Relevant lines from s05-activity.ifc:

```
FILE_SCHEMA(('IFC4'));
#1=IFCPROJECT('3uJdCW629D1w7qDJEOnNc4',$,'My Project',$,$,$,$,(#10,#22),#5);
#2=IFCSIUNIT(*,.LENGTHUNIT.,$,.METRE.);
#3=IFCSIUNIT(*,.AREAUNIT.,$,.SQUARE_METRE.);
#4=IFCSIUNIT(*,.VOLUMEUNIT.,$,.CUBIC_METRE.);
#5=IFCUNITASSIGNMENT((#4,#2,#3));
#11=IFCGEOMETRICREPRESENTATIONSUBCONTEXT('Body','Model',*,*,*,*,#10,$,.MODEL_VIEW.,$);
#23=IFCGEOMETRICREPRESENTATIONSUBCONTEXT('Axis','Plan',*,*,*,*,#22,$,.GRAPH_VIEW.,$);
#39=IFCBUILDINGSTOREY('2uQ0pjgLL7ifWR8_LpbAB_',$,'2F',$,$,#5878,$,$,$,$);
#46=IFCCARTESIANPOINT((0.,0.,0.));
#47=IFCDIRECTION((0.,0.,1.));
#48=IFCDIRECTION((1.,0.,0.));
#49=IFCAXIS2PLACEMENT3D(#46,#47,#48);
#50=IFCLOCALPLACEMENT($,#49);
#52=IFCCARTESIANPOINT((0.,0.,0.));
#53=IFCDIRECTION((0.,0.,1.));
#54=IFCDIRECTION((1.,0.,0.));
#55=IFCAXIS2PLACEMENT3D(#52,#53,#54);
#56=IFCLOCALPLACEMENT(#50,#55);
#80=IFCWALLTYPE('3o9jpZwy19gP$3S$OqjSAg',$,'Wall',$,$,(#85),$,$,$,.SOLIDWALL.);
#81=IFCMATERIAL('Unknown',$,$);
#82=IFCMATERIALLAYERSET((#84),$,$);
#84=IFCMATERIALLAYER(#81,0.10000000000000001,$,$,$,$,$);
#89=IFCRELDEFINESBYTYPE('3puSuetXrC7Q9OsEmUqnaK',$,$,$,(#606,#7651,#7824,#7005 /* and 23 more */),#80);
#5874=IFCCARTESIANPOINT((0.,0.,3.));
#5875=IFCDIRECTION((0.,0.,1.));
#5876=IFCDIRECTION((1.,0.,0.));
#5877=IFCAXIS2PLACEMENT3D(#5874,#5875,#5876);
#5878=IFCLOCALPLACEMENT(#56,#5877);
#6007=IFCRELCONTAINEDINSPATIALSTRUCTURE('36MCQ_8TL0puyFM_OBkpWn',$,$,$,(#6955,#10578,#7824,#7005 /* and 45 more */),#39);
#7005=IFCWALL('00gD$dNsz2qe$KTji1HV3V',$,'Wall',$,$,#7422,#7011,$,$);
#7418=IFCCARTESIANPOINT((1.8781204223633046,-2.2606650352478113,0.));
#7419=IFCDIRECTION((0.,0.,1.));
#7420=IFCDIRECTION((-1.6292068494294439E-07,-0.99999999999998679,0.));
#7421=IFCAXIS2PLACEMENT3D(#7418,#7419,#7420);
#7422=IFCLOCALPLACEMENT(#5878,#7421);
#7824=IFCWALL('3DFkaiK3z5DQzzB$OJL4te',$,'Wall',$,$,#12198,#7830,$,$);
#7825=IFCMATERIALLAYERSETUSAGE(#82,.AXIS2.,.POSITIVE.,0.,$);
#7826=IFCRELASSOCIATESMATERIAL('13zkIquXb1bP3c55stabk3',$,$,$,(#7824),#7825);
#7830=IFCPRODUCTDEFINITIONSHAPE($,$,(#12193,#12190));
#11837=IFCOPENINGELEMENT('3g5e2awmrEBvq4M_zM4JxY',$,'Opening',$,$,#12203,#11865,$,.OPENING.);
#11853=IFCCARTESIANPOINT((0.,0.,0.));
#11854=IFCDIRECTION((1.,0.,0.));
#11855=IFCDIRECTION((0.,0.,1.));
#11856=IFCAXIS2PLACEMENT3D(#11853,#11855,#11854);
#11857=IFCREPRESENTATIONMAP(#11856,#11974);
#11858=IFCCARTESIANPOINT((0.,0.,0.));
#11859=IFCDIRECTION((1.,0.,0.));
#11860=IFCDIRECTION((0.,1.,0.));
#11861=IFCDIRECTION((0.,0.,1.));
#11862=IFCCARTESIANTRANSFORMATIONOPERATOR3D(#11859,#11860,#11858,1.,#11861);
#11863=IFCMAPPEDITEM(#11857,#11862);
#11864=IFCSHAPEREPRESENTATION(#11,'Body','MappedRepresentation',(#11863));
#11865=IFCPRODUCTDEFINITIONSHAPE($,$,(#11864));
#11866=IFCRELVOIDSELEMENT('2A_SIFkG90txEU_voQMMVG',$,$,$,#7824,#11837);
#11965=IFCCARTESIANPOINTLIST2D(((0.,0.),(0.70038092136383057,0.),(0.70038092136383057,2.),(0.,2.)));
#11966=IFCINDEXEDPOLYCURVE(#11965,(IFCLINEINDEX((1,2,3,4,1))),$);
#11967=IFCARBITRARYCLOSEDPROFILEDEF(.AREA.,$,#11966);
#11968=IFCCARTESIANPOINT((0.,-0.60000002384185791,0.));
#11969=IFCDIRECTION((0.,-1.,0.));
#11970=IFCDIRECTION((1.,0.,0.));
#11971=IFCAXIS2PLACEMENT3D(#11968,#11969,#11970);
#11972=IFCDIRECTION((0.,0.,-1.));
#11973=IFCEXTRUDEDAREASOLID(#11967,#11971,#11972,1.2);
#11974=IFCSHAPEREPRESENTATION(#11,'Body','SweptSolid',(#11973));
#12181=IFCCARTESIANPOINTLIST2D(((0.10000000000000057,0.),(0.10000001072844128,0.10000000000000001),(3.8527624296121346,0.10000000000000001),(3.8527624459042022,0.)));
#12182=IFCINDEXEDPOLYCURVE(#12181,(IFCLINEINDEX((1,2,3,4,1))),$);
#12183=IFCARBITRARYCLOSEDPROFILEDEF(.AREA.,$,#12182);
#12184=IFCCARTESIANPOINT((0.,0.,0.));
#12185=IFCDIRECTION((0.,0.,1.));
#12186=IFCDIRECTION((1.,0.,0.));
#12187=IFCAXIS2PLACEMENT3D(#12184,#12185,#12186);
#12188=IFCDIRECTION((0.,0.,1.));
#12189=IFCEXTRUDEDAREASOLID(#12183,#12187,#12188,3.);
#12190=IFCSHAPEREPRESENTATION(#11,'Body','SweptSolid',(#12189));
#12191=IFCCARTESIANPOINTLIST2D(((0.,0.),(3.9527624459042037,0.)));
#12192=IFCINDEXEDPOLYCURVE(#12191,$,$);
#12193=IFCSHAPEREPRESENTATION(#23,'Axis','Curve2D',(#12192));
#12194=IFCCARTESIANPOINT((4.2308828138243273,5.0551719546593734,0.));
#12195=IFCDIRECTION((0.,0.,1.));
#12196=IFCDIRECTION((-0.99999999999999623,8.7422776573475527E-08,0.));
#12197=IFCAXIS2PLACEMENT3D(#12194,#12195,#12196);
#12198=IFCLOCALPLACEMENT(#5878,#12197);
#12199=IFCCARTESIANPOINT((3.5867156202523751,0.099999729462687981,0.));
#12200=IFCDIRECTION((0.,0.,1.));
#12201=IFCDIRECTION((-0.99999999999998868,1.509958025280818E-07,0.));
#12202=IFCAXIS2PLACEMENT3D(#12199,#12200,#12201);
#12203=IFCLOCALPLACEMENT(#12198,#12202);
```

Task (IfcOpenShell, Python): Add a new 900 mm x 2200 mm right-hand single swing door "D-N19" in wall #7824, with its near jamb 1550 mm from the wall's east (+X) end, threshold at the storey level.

```python
import numpy as np
import ifcopenshell
import ifcopenshell.api.feature
import ifcopenshell.api.geometry
import ifcopenshell.api.root
import ifcopenshell.api.spatial
import ifcopenshell.geom
import ifcopenshell.util.element
import ifcopenshell.util.placement
import ifcopenshell.util.representation
import ifcopenshell.util.shape
import ifcopenshell.util.unit

model = ifcopenshell.open("s05-activity.ifc")
unit_scale = ifcopenshell.util.unit.calculate_unit_scale(model)
settings = ifcopenshell.geom.settings()


def volume(element):
    """Net volume in cubic metres, openings subtracted."""
    shape = ifcopenshell.geom.create_shape(settings, element)
    return ifcopenshell.util.shape.get_volume(shape.geometry)


wall = model.by_guid("3DFkaiK3z5DQzzB$OJL4te")
storey = ifcopenshell.util.element.get_container(wall, ifc_class="IfcBuildingStorey")
context = ifcopenshell.util.representation.get_context(model, "Model", "Body", "MODEL_VIEW")
before = volume(wall)

width, height, from_end, sill = 0.9, 2.2, 1.55, 0.0  # metres

# The wall runs along its own X axis, and the end named is its -X end.
wall_shape = ifcopenshell.geom.create_shape(settings, wall)
x, y, z = ifcopenshell.util.shape.get_vertices(wall_shape.geometry).T
start = x.min() + from_end
face, thickness = float(y.min()), float(y.max() - y.min())
wall_matrix = ifcopenshell.util.placement.get_local_placement(wall.ObjectPlacement)
level = ifcopenshell.util.placement.get_local_placement(storey.ObjectPlacement)[2, 3]


def in_wall(x, y):
    """Placement at x, y metres in the wall's axes, at sill height."""
    matrix = wall_matrix.copy()
    matrix[:, 3] = wall_matrix @ np.array([x / unit_scale, y / unit_scale, 0.0, 1.0])
    matrix[2, 3] = level + sill / unit_scale
    return matrix


# Opening: a box that overshoots both wall faces by 50 mm.
opening = ifcopenshell.api.root.create_entity(model, ifc_class="IfcOpeningElement", predefined_type="OPENING")
box = ifcopenshell.api.geometry.add_wall_representation(
    model, context=context, length=width, height=height, thickness=thickness + 0.1
)
ifcopenshell.api.geometry.assign_representation(model, product=opening, representation=box)
ifcopenshell.api.geometry.edit_object_placement(model, product=opening, matrix=in_wall(start, face - 0.05), is_si=False)
ifcopenshell.api.feature.add_feature(model, feature=opening, element=wall)

door = ifcopenshell.api.root.create_entity(model, ifc_class="IfcDoor", name="D-N19", predefined_type="DOOR")
door.OverallWidth, door.OverallHeight = width / unit_scale, height / unit_scale
door.OperationType = "SINGLE_SWING_RIGHT"
body = ifcopenshell.api.geometry.add_door_representation(
    model,
    context=context,
    overall_width=door.OverallWidth,
    overall_height=door.OverallHeight,
    operation_type="SINGLE_SWING_RIGHT",
    lining_properties={"LiningDepth": thickness / unit_scale, "ThresholdDepth": thickness / unit_scale},
)
ifcopenshell.api.geometry.assign_representation(model, product=door, representation=body)
ifcopenshell.api.spatial.assign_container(model, products=[door], relating_structure=storey)
ifcopenshell.api.feature.add_filling(model, opening=opening, element=door)

# The lining spans the wall, so the door starts at the wall face.
ifcopenshell.api.geometry.edit_object_placement(model, product=door, matrix=in_wall(start, face), is_si=False)

after = volume(wall)

print(f"wall volume {before:.3f} -> {after:.3f} m3")

model.write("s05-activity_edited.ifc")
```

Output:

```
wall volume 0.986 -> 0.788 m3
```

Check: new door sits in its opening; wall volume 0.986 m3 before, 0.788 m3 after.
